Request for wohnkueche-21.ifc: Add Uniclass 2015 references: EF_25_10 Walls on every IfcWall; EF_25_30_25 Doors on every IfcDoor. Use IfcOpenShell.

First a look at what the model holds.

```python
import ifcopenshell

model = ifcopenshell.open("wohnkueche-21.ifc")
print(model.schema)
print("classifications:", [c.Name for c in model.by_type("IfcClassification")])
for ifc_class in ("IfcDoor", "IfcRoof", "IfcStair", "IfcWall", "IfcWindow"):
    print(ifc_class, len(model.by_type(ifc_class)))
```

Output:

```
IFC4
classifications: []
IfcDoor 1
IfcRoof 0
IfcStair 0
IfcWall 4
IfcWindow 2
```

```python
import ifcopenshell
import ifcopenshell.api.classification

model = ifcopenshell.open("wohnkueche-21.ifc")

system = ifcopenshell.api.classification.add_classification(model, classification="Uniclass 2015")

codes = {
    "IfcWall": ("EF_25_10", "Walls"),
    "IfcDoor": ("EF_25_30_25", "Doors"),
}
for ifc_class, (code, name) in codes.items():
    products = model.by_type(ifc_class)
    ifcopenshell.api.classification.add_reference(
        model, products=products, classification=system, identification=code, name=name
    )
    print(code, len(products))

model.write("wohnkueche-21_edited.ifc")
```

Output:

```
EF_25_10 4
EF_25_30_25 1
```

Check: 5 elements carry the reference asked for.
